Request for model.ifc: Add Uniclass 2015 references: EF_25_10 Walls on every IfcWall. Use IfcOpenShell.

First a look at what the model holds.

```python
import ifcopenshell

model = ifcopenshell.open("model.ifc")
print(model.schema)
print("classifications:", [c.Name for c in model.by_type("IfcClassification")])
for ifc_class in ("IfcDoor", "IfcRoof", "IfcStair", "IfcWall", "IfcWindow"):
    print(ifc_class, len(model.by_type(ifc_class)))
```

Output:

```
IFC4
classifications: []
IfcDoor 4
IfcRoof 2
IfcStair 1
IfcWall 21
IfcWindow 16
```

```python
import ifcopenshell
import ifcopenshell.api.classification

model = ifcopenshell.open("model.ifc")

system = ifcopenshell.api.classification.add_classification(model, classification="Uniclass 2015")

codes = {
    "IfcWall": ("EF_25_10", "Walls"),
}
for ifc_class, (code, name) in codes.items():
    products = model.by_type(ifc_class)
    ifcopenshell.api.classification.add_reference(
        model, products=products, classification=system, identification=code, name=name
    )
    print(code, len(products))

model.write("model_edited.ifc")
```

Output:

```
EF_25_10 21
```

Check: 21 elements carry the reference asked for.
